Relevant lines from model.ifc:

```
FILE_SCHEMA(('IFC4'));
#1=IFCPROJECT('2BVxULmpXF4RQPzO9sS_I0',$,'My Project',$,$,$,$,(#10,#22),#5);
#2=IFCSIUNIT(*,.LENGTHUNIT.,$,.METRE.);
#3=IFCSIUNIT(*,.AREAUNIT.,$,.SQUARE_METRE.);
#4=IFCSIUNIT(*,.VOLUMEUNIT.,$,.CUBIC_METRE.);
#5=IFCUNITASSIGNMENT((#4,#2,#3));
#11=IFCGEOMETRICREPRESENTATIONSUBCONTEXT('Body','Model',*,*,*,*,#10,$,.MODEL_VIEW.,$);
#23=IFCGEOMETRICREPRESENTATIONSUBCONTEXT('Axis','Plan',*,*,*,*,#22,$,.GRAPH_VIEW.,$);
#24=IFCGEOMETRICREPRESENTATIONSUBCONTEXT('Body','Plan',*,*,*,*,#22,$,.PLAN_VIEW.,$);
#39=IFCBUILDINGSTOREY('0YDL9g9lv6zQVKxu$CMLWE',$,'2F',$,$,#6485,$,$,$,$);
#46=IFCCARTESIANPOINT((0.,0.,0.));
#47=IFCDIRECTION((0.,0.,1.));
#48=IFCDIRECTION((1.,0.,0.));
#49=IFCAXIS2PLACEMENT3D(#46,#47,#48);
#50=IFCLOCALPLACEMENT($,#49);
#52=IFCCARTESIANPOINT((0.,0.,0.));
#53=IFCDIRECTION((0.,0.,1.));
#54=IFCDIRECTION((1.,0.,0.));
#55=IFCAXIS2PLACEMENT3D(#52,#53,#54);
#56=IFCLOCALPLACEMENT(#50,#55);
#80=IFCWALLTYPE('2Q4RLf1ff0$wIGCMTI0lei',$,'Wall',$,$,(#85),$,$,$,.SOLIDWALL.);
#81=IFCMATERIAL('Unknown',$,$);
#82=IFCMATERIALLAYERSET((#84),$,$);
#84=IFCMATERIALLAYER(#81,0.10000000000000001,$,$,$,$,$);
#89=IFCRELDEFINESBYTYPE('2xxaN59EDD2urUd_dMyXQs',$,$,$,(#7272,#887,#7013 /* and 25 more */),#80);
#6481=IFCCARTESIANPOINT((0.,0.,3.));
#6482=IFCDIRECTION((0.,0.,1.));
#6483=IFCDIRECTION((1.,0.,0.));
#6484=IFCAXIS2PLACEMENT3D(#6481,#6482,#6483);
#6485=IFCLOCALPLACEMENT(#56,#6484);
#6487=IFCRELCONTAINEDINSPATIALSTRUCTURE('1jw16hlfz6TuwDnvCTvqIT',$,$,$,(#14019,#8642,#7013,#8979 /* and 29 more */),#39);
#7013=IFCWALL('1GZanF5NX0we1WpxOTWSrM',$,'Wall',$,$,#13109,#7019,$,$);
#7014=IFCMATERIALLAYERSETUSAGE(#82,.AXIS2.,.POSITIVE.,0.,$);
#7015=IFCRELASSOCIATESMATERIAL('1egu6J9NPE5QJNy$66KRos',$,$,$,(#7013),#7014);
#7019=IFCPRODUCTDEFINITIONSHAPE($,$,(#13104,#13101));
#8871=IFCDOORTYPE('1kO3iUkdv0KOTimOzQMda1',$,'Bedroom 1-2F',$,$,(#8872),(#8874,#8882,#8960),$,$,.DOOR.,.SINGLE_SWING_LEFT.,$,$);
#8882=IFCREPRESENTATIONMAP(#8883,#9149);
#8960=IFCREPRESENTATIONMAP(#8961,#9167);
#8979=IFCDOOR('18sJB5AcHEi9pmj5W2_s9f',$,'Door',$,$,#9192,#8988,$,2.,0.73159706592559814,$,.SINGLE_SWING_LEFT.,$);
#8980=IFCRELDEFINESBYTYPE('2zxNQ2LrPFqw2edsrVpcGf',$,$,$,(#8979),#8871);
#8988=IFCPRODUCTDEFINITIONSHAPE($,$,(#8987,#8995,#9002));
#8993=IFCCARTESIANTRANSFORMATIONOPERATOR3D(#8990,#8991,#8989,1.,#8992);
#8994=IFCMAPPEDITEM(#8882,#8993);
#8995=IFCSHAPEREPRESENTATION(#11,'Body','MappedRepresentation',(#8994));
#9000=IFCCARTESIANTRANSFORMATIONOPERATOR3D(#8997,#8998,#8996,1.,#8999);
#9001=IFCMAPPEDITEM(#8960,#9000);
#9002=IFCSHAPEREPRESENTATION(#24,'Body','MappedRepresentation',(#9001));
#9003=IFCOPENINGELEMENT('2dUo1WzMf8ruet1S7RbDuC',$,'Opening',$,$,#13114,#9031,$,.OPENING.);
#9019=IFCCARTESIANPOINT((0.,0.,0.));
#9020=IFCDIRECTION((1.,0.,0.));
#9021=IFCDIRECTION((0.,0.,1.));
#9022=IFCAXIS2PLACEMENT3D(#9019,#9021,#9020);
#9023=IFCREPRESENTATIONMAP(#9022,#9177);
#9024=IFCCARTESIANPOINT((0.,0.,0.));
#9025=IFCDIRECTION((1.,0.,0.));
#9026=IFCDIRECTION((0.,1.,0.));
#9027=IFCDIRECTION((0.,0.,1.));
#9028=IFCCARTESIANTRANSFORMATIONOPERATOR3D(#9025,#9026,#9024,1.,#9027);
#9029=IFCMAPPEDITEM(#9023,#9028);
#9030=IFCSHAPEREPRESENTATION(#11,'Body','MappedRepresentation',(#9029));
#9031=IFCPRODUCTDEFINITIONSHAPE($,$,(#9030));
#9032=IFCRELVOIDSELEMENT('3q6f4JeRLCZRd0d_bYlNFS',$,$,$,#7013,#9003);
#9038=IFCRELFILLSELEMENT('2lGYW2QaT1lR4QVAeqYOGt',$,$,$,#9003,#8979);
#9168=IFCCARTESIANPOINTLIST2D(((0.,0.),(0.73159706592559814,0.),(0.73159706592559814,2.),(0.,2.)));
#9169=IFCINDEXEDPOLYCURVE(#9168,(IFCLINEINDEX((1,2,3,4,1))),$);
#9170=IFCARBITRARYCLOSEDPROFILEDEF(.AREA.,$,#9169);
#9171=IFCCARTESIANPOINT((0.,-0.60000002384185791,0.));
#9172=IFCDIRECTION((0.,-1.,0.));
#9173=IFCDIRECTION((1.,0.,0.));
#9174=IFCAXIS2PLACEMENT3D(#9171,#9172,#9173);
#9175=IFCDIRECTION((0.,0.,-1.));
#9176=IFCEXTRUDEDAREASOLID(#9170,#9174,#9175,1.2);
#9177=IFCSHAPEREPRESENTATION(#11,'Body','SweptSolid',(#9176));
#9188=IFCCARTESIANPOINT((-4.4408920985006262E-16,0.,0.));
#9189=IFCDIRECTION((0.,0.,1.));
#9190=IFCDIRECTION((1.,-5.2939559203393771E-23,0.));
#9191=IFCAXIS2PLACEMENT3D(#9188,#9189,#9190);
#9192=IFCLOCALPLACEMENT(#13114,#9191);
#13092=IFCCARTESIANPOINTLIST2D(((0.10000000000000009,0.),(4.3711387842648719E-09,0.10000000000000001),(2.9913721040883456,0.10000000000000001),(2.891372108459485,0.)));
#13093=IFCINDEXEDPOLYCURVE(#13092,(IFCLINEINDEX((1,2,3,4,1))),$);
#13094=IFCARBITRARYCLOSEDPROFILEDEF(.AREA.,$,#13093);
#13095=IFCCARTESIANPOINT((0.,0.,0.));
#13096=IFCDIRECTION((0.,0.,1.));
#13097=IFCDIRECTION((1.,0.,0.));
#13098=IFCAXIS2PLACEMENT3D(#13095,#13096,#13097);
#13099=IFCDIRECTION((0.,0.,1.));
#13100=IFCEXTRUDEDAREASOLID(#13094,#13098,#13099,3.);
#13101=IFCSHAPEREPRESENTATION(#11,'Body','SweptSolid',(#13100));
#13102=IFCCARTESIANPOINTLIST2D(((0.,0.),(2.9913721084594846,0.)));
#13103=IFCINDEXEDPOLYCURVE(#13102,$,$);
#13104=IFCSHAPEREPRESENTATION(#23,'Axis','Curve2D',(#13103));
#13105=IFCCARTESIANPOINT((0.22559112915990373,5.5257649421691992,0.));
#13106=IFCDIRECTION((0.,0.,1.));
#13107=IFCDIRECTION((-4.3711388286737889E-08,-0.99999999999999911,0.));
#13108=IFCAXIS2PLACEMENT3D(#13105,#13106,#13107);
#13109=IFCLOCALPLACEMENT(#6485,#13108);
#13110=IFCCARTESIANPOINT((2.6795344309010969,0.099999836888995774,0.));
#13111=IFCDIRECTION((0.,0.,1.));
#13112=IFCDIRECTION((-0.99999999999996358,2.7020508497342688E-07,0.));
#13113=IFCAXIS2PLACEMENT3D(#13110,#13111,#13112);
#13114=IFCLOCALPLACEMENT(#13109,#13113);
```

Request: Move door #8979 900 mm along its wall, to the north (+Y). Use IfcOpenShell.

```python
import ifcopenshell
import ifcopenshell.api.geometry
import ifcopenshell.util.placement
import ifcopenshell.util.unit

model = ifcopenshell.open("model.ifc")
unit_scale = ifcopenshell.util.unit.calculate_unit_scale(model)

door = model.by_id(8979)
opening = door.FillsVoids[0].RelatingOpeningElement
wall = opening.VoidsElements[0].RelatingBuildingElement

wall_matrix = ifcopenshell.util.placement.get_local_placement(wall.ObjectPlacement)
shift = wall_matrix[:3, 0] * -0.9 / unit_scale
before = ifcopenshell.util.placement.get_local_placement(door.ObjectPlacement)[:3, 3].copy()

# The door is placed relative to its opening, so it follows when the opening moves.
matrix = ifcopenshell.util.placement.get_local_placement(opening.ObjectPlacement)
matrix[:3, 3] += shift
ifcopenshell.api.geometry.edit_object_placement(
    model, product=opening, matrix=matrix, is_si=False, should_transform_children=True
)

after = ifcopenshell.util.placement.get_local_placement(door.ObjectPlacement)[:3, 3]
print("door moved by", (after - before).round(3) + 0.0)

model.write("model-out.ifc")
```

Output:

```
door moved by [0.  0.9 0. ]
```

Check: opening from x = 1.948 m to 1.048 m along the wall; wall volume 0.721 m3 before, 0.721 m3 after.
